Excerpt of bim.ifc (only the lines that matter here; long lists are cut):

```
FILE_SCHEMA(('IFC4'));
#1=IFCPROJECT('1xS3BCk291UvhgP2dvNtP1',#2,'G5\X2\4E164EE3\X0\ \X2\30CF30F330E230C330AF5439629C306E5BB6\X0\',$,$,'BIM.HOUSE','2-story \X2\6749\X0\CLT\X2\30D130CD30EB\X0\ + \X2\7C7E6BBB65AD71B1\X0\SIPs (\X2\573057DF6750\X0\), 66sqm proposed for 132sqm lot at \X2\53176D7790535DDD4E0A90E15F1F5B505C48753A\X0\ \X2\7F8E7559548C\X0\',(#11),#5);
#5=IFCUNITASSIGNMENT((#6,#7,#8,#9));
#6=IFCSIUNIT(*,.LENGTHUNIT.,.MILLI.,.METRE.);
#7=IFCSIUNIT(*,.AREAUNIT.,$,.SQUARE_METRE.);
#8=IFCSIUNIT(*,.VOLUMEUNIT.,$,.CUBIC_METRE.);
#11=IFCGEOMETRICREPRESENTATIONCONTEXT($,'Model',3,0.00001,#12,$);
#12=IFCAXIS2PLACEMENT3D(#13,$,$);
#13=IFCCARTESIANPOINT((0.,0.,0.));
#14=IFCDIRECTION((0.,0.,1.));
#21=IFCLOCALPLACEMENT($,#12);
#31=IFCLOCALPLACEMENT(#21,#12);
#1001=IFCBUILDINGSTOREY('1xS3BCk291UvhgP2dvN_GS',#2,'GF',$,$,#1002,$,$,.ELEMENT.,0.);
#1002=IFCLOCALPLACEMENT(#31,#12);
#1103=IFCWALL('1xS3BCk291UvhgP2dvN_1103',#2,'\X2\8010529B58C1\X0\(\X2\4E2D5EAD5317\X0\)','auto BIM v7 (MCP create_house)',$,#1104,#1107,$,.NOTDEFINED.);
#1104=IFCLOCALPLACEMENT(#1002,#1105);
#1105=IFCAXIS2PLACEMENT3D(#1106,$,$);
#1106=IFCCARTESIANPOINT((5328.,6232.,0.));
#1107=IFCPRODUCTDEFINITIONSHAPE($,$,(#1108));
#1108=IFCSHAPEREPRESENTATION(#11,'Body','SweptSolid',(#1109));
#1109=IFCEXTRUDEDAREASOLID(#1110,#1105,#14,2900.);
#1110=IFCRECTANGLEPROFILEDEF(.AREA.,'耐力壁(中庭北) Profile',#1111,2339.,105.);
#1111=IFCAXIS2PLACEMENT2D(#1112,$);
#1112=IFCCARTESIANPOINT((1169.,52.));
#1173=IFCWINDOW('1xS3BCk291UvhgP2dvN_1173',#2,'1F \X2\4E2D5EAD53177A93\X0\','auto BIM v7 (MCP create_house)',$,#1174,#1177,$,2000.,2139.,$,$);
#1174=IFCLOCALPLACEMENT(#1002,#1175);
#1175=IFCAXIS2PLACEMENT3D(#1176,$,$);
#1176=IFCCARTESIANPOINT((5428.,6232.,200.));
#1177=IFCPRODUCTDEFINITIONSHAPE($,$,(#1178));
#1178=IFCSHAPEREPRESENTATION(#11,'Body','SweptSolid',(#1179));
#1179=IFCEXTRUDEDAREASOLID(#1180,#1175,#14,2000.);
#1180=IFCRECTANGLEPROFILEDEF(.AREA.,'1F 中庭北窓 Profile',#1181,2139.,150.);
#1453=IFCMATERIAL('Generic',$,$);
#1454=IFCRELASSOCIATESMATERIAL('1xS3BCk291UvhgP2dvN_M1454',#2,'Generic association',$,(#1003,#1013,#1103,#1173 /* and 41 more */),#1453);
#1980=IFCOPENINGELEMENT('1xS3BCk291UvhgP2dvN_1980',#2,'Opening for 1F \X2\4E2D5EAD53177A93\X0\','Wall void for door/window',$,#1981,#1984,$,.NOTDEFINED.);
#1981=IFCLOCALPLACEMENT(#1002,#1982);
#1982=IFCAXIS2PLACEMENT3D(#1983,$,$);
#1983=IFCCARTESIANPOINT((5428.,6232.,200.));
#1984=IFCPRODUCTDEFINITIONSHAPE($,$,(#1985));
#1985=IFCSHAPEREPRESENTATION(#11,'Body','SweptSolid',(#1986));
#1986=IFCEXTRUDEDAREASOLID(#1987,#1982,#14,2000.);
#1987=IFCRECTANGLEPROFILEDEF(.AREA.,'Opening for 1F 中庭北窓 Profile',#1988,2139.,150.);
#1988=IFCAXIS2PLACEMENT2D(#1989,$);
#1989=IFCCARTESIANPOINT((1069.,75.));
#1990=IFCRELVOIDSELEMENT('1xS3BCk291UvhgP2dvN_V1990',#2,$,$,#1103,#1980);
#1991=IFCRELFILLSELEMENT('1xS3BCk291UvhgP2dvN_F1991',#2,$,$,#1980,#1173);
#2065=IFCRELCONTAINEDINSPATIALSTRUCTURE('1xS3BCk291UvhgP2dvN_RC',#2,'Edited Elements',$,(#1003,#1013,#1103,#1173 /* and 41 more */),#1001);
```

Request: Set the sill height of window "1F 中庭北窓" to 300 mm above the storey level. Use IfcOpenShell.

```python
import numpy as np
import ifcopenshell
import ifcopenshell.api.geometry
import ifcopenshell.geom
import ifcopenshell.util.element
import ifcopenshell.util.placement
import ifcopenshell.util.shape
import ifcopenshell.util.unit

model = ifcopenshell.open("bim.ifc")
unit_scale = ifcopenshell.util.unit.calculate_unit_scale(model)

window = model.by_id(1173)
opening = window.FillsVoids[0].RelatingOpeningElement
storey = ifcopenshell.util.element.get_container(window, ifc_class="IfcBuildingStorey")
level = ifcopenshell.util.placement.get_local_placement(storey.ObjectPlacement)[2, 3]

# The opening's origin need not be at the sill, so measure its lowest point.
shape = ifcopenshell.geom.create_shape(ifcopenshell.geom.settings(), opening)
bottom = ifcopenshell.util.shape.get_shape_bottom_elevation(shape, shape.geometry) / unit_scale
dz = level + 0.3 / unit_scale - bottom

shift = np.array([0.0, 0.0, dz])
# The window is not placed relative to its opening, so move both.
for product in (opening, window):
    matrix = ifcopenshell.util.placement.get_local_placement(product.ObjectPlacement)
    matrix[:3, 3] += shift
    ifcopenshell.api.geometry.edit_object_placement(model, product=product, matrix=matrix, is_si=False)

print(f"moved by {dz * unit_scale:+.3f} m")

model.write("bim_updated.ifc")
```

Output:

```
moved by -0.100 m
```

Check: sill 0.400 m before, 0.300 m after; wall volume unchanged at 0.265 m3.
